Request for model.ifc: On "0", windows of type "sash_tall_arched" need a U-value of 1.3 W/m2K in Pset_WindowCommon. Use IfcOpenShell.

First a look at what the model holds.

```python
import ifcopenshell
import ifcopenshell.util.element

model = ifcopenshell.open("model.ifc")
print(model.schema)
storey = next(s for s in model.by_type("IfcBuildingStorey") if s.Name == "0")
windows = [e for e in ifcopenshell.util.element.get_decomposition(storey) if e.is_a("IfcWindow")]
seen = {}
for e in windows:
    element_type = ifcopenshell.util.element.get_type(e)
    key = (element_type.Name if element_type != e and element_type else None, ifcopenshell.util.element.get_pset(e, "Pset_WindowCommon", "ThermalTransmittance"))
    seen[key] = seen.get(key, 0) + 1
for (name, value), count in sorted(seen.items(), key=str):
    print(count, "x", name, "|", value)
```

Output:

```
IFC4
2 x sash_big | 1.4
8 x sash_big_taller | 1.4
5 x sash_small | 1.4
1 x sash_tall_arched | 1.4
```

```python
import ifcopenshell
import ifcopenshell.api.pset
import ifcopenshell.util.element

model = ifcopenshell.open("model.ifc")

storey = next(s for s in model.by_type("IfcBuildingStorey") if s.Name == "0")
windows = [e for e in ifcopenshell.util.element.get_decomposition(storey) if e.is_a("IfcWindow")]

count = 0
for e in windows:
    element_type = ifcopenshell.util.element.get_type(e)
    if element_type in (None, e) or element_type.Name != "sash_tall_arched":
        continue
    # add_pset returns the element's existing set when there is one.
    pset = ifcopenshell.api.pset.add_pset(model, product=e, name="Pset_WindowCommon")
    ifcopenshell.api.pset.edit_pset(model, pset=pset, properties={"ThermalTransmittance": 1.3})
    count += 1

print(count, "windows updated")

model.write("model_updated.ifc")
```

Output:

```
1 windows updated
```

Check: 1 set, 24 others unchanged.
